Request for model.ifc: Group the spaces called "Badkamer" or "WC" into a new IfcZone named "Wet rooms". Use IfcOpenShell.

First a look at what the model holds.

```python
import ifcopenshell

model = ifcopenshell.open("model.ifc")
print(model.schema)
seen = {}
for space in model.by_type("IfcSpace"):
    seen[space.LongName] = seen.get(space.LongName, 0) + 1
for name, count in sorted(seen.items(), key=str):
    print(count, "x", name)
print("zones:", [z.Name for z in model.by_type("IfcZone")][:20])
```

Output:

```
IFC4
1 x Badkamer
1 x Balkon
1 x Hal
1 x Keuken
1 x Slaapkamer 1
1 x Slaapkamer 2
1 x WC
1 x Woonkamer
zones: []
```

```python
import ifcopenshell
import ifcopenshell.api.group
import ifcopenshell.api.root

model = ifcopenshell.open("model.ifc")

names = {"Badkamer", "WC"}
spaces = [s for s in model.by_type("IfcSpace") if s.LongName in names]

zone = ifcopenshell.api.root.create_entity(model, ifc_class="IfcZone", name="Wet rooms")
ifcopenshell.api.group.assign_group(model, products=spaces, group=zone)
print(len(spaces), "spaces in", zone.Name)

model.write("model_updated.ifc")
```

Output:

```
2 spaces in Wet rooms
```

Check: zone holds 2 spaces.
